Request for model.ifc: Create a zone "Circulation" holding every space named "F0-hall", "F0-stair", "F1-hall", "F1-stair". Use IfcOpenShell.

First a look at what the model holds.

```python
import ifcopenshell

model = ifcopenshell.open("model.ifc")
print(model.schema)
seen = {}
for space in model.by_type("IfcSpace"):
    seen[space.LongName] = seen.get(space.LongName, 0) + 1
for name, count in sorted(seen.items(), key=str):
    print(count, "x", name)
print("zones:", [z.Name for z in model.by_type("IfcZone")][:20])
```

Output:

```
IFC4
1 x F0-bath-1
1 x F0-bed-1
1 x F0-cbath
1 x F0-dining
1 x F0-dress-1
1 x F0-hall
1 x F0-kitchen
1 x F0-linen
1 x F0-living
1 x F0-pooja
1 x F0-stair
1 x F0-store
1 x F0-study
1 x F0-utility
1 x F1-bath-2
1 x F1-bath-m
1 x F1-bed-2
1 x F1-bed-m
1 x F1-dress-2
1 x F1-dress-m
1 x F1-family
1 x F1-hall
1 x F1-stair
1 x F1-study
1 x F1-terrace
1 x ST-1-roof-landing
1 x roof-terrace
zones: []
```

```python
import ifcopenshell
import ifcopenshell.api.group
import ifcopenshell.api.root

model = ifcopenshell.open("model.ifc")

names = {"F0-hall", "F0-stair", "F1-hall", "F1-stair"}
spaces = [s for s in model.by_type("IfcSpace") if s.LongName in names]

zone = ifcopenshell.api.root.create_entity(model, ifc_class="IfcZone", name="Circulation")
ifcopenshell.api.group.assign_group(model, products=spaces, group=zone)
print(len(spaces), "spaces in", zone.Name)

model.write("model_updated.ifc")
```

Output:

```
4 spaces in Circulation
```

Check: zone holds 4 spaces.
